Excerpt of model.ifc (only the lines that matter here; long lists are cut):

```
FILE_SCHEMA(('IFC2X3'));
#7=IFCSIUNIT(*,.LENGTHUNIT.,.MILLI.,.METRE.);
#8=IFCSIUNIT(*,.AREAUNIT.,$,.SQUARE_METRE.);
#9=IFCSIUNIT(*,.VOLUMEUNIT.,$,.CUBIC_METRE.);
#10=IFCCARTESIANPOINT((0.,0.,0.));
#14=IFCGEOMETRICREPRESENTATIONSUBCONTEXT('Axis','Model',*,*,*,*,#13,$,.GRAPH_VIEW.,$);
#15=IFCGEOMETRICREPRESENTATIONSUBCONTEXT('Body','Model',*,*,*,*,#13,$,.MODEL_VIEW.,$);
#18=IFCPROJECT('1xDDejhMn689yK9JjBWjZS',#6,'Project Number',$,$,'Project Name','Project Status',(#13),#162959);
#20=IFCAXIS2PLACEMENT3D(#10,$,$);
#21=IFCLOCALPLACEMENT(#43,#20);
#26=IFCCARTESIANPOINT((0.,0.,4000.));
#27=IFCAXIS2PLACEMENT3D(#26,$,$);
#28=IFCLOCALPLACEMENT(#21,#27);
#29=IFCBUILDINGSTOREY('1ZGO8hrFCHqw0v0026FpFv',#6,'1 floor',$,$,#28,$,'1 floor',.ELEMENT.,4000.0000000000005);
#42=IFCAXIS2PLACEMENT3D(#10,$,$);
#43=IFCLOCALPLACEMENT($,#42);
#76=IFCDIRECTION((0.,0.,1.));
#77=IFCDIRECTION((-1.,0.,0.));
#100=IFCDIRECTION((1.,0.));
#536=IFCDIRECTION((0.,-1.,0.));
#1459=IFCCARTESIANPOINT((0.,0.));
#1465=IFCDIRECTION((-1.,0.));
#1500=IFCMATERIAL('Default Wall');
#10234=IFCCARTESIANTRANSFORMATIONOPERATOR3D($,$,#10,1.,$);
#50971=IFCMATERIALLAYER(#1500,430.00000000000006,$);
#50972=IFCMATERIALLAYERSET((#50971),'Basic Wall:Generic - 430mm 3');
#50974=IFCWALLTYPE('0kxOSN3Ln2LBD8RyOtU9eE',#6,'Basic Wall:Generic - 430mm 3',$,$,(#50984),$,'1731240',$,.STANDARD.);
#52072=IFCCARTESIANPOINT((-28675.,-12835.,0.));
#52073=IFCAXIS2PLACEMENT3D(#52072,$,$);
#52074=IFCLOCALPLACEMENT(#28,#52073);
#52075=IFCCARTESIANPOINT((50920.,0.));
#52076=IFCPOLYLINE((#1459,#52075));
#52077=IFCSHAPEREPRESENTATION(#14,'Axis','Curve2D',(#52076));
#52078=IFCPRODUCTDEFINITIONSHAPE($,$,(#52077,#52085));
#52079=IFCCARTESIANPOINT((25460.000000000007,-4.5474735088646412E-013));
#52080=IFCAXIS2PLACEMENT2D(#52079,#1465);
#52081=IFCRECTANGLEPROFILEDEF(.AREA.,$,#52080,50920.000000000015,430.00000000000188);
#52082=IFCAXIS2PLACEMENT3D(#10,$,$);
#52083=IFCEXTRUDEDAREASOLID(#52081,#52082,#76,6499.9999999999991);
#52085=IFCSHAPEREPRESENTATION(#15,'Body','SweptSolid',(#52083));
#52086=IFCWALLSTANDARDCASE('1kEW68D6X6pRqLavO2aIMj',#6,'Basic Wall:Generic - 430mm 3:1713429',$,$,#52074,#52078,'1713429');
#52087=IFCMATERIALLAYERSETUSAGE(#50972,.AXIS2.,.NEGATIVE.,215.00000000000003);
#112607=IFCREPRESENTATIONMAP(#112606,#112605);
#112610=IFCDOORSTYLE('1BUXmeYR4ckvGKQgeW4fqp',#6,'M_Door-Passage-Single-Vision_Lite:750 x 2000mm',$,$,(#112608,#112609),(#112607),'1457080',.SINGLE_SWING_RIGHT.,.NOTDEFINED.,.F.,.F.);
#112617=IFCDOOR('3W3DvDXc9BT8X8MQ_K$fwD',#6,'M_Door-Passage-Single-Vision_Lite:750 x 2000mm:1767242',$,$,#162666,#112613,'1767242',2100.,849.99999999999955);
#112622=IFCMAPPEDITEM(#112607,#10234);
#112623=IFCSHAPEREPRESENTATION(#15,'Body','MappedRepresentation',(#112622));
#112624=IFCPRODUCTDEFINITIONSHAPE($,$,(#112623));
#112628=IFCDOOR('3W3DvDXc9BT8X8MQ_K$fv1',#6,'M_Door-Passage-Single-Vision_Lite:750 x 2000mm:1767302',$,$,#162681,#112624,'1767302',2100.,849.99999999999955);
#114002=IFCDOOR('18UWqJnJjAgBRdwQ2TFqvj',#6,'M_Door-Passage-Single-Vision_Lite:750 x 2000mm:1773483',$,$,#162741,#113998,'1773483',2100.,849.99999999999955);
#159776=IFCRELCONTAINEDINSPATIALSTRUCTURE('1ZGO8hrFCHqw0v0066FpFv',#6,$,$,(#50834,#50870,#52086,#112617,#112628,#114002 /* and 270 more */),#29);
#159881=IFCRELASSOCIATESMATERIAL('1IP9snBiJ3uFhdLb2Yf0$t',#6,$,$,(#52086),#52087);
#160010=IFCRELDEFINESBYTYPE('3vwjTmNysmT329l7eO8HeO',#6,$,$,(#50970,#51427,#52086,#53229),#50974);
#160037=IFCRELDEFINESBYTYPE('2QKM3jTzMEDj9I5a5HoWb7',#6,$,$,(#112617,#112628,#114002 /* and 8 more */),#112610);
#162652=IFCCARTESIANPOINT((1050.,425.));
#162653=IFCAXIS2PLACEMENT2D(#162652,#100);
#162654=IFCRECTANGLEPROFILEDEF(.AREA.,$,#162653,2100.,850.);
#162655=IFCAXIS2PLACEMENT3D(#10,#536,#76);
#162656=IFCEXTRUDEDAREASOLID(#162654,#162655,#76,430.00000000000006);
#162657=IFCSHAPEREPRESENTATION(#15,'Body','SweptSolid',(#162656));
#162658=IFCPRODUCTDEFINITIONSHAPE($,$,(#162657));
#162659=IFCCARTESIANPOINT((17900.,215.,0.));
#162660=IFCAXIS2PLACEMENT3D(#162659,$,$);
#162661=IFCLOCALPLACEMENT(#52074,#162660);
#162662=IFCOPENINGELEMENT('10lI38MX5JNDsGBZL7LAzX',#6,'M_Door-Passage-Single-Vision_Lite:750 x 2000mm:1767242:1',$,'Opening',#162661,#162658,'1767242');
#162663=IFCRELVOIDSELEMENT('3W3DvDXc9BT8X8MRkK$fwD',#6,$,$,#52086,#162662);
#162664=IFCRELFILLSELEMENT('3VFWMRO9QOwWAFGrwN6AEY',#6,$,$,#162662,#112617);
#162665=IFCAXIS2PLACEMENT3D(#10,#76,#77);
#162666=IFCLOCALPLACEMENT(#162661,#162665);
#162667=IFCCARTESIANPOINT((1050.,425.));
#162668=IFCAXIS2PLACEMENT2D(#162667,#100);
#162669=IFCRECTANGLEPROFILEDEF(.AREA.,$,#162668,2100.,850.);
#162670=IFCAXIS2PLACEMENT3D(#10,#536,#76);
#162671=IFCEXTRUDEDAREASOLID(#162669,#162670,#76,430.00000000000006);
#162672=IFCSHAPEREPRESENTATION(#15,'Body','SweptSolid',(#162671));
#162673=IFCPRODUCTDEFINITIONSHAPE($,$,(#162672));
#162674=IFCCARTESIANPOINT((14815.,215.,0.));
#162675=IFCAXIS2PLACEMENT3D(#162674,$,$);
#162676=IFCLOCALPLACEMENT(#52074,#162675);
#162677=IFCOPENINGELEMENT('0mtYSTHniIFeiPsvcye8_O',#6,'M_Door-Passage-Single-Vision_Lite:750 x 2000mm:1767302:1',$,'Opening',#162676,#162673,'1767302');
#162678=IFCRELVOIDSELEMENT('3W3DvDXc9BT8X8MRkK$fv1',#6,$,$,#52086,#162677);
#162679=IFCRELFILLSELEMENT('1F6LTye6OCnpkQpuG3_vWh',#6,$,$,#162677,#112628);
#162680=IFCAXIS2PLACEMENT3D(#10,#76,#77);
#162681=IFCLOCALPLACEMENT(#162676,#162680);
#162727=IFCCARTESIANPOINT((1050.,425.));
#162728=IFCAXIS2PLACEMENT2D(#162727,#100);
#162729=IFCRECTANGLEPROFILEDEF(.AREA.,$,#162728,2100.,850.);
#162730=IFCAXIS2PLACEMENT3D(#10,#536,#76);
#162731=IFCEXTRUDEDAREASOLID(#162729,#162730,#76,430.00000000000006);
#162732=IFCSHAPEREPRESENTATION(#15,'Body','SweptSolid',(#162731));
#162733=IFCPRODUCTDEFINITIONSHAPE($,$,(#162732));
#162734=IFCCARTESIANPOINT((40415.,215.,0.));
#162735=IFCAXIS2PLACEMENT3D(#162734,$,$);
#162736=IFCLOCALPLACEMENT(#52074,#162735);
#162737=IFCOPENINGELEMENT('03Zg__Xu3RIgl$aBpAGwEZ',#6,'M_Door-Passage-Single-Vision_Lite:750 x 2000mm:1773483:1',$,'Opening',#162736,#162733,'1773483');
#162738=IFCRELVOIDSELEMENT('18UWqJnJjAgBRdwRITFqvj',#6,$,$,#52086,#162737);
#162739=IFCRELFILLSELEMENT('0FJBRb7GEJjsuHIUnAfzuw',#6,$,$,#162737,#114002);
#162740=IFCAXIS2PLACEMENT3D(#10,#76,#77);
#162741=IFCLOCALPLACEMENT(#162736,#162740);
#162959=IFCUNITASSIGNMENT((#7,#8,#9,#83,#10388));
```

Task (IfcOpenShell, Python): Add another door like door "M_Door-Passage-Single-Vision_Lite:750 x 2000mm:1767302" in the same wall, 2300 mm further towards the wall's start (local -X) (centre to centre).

```python
import ifcopenshell
import ifcopenshell.api.feature
import ifcopenshell.api.geometry
import ifcopenshell.api.root
import ifcopenshell.geom
import ifcopenshell.util.element
import ifcopenshell.util.placement
import ifcopenshell.util.shape
import ifcopenshell.util.unit

model = ifcopenshell.open("model.ifc")
unit_scale = ifcopenshell.util.unit.calculate_unit_scale(model)
settings = ifcopenshell.geom.settings()


def volume(element):
    """Net volume in cubic metres, openings subtracted."""
    shape = ifcopenshell.geom.create_shape(settings, element)
    return ifcopenshell.util.shape.get_volume(shape.geometry)


def reuse_history(source, copy):
    """copy_class also copies each property set's owner history, people and application; keep the originals."""
    for rel in copy.IsDefinedBy:
        if rel.is_a("IfcRelDefinesByProperties") and (history := rel.RelatingPropertyDefinition.OwnerHistory):
            rel.RelatingPropertyDefinition.OwnerHistory = source.OwnerHistory
            ifcopenshell.util.element.remove_deep2(model, history)


door = model.by_id(112628)
opening = door.FillsVoids[0].RelatingOpeningElement
wall = opening.VoidsElements[0].RelatingBuildingElement
before = volume(wall)
shift = ifcopenshell.util.placement.get_local_placement(wall.ObjectPlacement)[:3, 0] * -2.3 / unit_scale

# copy_class copies the void relationship, type, container and properties, but no geometry.
new_opening = ifcopenshell.api.root.copy_class(model, product=opening)
new_opening.Representation = ifcopenshell.util.element.copy_deep(
    model, opening.Representation, exclude=["IfcGeometricRepresentationContext", "IfcRepresentationMap"]
)
new_opening.Name = "M_Door-Passage-Single-Vision_Lite:750 x 2000mm"
new_opening.Tag = None
new_door = ifcopenshell.api.root.copy_class(model, product=door)
new_door.Representation = ifcopenshell.util.element.copy_deep(
    model, door.Representation, exclude=["IfcGeometricRepresentationContext", "IfcRepresentationMap"]
)
new_door.Name = "M_Door-Passage-Single-Vision_Lite:750 x 2000mm"
new_door.Tag = None
reuse_history(door, new_door)
fills = ifcopenshell.api.feature.add_filling(model, opening=new_opening, element=new_door)
fills.OwnerHistory = new_door.OwnerHistory  # required in IFC2X3

for old, new in ((opening, new_opening), (door, new_door)):
    matrix = ifcopenshell.util.placement.get_local_placement(old.ObjectPlacement)
    matrix[:3, 3] += shift
    ifcopenshell.api.geometry.edit_object_placement(model, product=new, matrix=matrix, is_si=False)

after = volume(wall)

print(f"wall volume {before:.3f} -> {after:.3f} m3")

model.write("model_edited.ifc")
```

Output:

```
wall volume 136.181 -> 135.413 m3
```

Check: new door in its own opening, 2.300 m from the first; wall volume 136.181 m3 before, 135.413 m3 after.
